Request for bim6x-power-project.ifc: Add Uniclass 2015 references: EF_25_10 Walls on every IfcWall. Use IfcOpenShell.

First a look at what the model holds.

```python
import ifcopenshell

model = ifcopenshell.open("bim6x-power-project.ifc")
print(model.schema)
print("classifications:", [c.Name for c in model.by_type("IfcClassification")])
for ifc_class in ("IfcDoor", "IfcRoof", "IfcStair", "IfcWall", "IfcWindow"):
    print(ifc_class, len(model.by_type(ifc_class)))
```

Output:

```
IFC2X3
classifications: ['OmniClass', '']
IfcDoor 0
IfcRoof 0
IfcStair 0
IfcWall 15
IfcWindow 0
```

```python
import ifcopenshell
import ifcopenshell.api.classification

model = ifcopenshell.open("bim6x-power-project.ifc")

# IFC2X3 requires Source and Edition and has no link from the project to the system.
system = model.create_entity("IfcClassification", Source="NBS", Edition="2015", Name="Uniclass 2015")

codes = {
    "IfcWall": ("EF_25_10", "Walls"),
}
for ifc_class, (code, name) in codes.items():
    products = model.by_type(ifc_class)
    ifcopenshell.api.classification.add_reference(
        model, products=products, classification=system, identification=code, name=name
    )
    print(code, len(products))

model.write("bim6x-power-project-out.ifc")
```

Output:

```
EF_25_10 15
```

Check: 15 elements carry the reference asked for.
